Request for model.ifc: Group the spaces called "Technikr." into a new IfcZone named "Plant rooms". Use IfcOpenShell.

First a look at what the model holds.

```python
import ifcopenshell

model = ifcopenshell.open("model.ifc")
print(model.schema)
seen = {}
for space in model.by_type("IfcSpace"):
    seen[space.LongName] = seen.get(space.LongName, 0) + 1
for name, count in sorted(seen.items(), key=str):
    print(count, "x", name)
print("zones:", [z.Name for z in model.by_type("IfcZone")][:20])
```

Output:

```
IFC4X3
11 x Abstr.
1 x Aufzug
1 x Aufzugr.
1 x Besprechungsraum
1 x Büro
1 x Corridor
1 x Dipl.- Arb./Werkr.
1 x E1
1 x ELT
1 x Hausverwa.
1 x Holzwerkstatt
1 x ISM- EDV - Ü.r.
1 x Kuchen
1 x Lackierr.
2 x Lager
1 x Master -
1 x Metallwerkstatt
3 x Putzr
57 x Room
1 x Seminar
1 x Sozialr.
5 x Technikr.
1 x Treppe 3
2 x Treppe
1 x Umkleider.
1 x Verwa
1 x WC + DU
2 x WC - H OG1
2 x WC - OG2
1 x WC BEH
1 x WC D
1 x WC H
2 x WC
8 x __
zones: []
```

```python
import ifcopenshell
import ifcopenshell.api.group
import ifcopenshell.api.root

model = ifcopenshell.open("model.ifc")

names = {"Technikr."}
spaces = [s for s in model.by_type("IfcSpace") if s.LongName in names]

zone = ifcopenshell.api.root.create_entity(model, ifc_class="IfcZone", name="Plant rooms")
ifcopenshell.api.group.assign_group(model, products=spaces, group=zone)
print(len(spaces), "spaces in", zone.Name)

model.write("model_v2.ifc")
```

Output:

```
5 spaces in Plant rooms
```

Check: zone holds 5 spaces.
